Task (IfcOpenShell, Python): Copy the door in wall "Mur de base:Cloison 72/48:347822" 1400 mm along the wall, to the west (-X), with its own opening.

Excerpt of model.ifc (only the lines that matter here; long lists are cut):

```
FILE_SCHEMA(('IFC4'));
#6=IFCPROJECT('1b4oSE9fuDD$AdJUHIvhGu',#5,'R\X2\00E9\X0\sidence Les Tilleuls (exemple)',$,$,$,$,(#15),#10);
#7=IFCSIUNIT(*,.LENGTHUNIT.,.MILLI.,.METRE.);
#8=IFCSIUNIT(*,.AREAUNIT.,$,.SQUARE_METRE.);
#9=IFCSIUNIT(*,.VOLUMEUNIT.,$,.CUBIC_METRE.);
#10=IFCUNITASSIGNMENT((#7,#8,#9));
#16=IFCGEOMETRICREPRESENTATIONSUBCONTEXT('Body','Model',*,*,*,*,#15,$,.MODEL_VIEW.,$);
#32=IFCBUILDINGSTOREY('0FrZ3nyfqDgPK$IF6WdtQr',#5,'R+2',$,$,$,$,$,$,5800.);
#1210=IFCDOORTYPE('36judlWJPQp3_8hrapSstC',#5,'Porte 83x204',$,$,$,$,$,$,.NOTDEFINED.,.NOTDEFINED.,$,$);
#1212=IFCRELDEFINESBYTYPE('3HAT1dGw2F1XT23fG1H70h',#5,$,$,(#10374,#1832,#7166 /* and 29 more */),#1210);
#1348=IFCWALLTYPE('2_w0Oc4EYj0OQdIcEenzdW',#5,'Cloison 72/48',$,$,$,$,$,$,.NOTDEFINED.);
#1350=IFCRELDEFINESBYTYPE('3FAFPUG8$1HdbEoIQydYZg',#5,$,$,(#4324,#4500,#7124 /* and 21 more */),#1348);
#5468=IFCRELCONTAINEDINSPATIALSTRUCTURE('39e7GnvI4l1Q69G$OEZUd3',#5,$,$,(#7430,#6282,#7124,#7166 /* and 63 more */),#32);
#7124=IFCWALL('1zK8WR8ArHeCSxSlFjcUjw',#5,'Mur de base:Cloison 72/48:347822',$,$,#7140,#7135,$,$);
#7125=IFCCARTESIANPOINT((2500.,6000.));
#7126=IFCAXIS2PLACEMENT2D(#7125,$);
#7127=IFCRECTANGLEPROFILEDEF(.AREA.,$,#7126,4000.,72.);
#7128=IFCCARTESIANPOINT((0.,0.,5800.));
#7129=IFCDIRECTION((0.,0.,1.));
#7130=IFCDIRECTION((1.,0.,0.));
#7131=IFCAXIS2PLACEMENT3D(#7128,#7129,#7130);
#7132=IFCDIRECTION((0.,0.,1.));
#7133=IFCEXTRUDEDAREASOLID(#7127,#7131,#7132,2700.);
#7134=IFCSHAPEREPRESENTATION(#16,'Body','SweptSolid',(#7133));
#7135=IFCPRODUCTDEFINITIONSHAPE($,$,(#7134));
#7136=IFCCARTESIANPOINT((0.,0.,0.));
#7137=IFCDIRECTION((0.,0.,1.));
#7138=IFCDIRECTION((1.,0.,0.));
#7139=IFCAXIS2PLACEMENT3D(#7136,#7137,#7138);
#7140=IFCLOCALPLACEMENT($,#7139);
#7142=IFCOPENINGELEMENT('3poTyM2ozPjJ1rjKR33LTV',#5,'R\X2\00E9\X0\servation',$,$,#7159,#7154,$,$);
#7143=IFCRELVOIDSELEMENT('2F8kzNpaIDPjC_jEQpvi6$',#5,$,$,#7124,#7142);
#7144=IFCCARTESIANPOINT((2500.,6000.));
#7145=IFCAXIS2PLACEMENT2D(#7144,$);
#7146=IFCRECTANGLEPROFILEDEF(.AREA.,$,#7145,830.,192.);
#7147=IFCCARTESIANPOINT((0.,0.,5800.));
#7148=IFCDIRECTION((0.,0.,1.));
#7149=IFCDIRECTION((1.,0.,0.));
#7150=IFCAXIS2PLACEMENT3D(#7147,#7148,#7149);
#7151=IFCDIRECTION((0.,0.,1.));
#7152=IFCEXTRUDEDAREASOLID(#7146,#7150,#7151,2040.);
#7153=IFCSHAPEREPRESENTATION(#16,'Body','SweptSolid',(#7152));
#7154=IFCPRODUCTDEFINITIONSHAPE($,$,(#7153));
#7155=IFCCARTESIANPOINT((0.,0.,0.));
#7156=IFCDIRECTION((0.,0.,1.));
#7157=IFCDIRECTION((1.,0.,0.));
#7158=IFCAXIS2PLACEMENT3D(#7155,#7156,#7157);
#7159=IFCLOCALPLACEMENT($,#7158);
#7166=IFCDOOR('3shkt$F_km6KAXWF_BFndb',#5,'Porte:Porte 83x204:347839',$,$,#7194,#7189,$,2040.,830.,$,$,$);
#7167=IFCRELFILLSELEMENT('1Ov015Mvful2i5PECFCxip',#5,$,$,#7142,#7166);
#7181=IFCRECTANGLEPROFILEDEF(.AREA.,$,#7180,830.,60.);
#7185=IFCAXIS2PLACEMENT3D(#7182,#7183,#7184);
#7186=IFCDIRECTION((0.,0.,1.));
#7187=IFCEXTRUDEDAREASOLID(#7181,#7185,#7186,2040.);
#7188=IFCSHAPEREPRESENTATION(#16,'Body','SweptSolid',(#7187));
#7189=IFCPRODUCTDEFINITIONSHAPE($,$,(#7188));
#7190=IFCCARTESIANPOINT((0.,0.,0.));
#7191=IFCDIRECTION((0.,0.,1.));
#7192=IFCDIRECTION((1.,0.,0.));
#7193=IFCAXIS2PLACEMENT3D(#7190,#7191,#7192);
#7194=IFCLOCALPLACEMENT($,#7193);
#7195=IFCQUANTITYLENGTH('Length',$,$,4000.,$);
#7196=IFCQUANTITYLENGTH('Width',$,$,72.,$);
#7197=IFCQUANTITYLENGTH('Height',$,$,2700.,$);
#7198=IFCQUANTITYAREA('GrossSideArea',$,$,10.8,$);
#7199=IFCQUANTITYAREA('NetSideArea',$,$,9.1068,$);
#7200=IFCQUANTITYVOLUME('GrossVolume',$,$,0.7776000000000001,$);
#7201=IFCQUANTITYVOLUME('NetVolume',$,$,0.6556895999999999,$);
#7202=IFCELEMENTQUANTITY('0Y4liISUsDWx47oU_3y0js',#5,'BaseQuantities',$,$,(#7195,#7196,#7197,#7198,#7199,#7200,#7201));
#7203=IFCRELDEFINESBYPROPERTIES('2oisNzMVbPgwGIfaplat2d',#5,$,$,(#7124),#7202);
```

```python
import ifcopenshell
import ifcopenshell.api.feature
import ifcopenshell.api.geometry
import ifcopenshell.api.pset
import ifcopenshell.api.root
import ifcopenshell.geom
import ifcopenshell.util.element
import ifcopenshell.util.placement
import ifcopenshell.util.shape
import ifcopenshell.util.unit

model = ifcopenshell.open("model.ifc")
area_scale = ifcopenshell.util.unit.calculate_unit_scale(model, "AREAUNIT")
volume_scale = ifcopenshell.util.unit.calculate_unit_scale(model, "VOLUMEUNIT")
settings = ifcopenshell.geom.settings()


def volume(element):
    """Net volume in cubic metres, openings subtracted."""
    shape = ifcopenshell.geom.create_shape(settings, element)
    return ifcopenshell.util.shape.get_volume(shape.geometry)


def reuse_history(source, copy):
    """copy_class also copies each property set's owner history, people and application; keep the originals."""
    for rel in copy.IsDefinedBy:
        if rel.is_a("IfcRelDefinesByProperties") and (history := rel.RelatingPropertyDefinition.OwnerHistory):
            rel.RelatingPropertyDefinition.OwnerHistory = source.OwnerHistory
            ifcopenshell.util.element.remove_deep2(model, history)


door = model.by_id(7166)
opening = door.FillsVoids[0].RelatingOpeningElement
wall = opening.VoidsElements[0].RelatingBuildingElement
before = volume(wall)
shift = ifcopenshell.util.placement.get_local_placement(wall.ObjectPlacement)[:3, 0] * -1400.0

# copy_class copies the void relationship, type, container and properties, but no geometry.
new_opening = ifcopenshell.api.root.copy_class(model, product=opening)
new_opening.Representation = ifcopenshell.util.element.copy_deep(
    model, opening.Representation, exclude=["IfcGeometricRepresentationContext", "IfcRepresentationMap"]
)
reuse_history(opening, new_opening)
new_door = ifcopenshell.api.root.copy_class(model, product=door)
new_door.Representation = ifcopenshell.util.element.copy_deep(
    model, door.Representation, exclude=["IfcGeometricRepresentationContext", "IfcRepresentationMap"]
)
new_door.Name = "Porte:Porte 83x204"
reuse_history(door, new_door)
ifcopenshell.api.feature.add_filling(model, opening=new_opening, element=new_door)

for old, new in ((opening, new_opening), (door, new_door)):
    matrix = ifcopenshell.util.placement.get_local_placement(old.ObjectPlacement)
    matrix[:3, 3] += shift
    ifcopenshell.api.geometry.edit_object_placement(model, product=new, matrix=matrix, is_si=False)

after = volume(wall)
thickness = 0.072  # wall thickness in metres

# Update the wall's stored quantities.
qto = model.by_id(ifcopenshell.util.element.get_pset(wall, "BaseQuantities", should_inherit=False)["id"])
ifcopenshell.api.pset.edit_qto(model, qto=qto, properties={
    "NetSideArea": after / thickness / area_scale,
    "NetVolume": after / volume_scale,
})

print(f"wall volume {before:.3f} -> {after:.3f} m3")

model.write("model_edited.ifc")
```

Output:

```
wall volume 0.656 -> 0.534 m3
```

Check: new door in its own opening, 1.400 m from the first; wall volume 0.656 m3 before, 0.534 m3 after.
